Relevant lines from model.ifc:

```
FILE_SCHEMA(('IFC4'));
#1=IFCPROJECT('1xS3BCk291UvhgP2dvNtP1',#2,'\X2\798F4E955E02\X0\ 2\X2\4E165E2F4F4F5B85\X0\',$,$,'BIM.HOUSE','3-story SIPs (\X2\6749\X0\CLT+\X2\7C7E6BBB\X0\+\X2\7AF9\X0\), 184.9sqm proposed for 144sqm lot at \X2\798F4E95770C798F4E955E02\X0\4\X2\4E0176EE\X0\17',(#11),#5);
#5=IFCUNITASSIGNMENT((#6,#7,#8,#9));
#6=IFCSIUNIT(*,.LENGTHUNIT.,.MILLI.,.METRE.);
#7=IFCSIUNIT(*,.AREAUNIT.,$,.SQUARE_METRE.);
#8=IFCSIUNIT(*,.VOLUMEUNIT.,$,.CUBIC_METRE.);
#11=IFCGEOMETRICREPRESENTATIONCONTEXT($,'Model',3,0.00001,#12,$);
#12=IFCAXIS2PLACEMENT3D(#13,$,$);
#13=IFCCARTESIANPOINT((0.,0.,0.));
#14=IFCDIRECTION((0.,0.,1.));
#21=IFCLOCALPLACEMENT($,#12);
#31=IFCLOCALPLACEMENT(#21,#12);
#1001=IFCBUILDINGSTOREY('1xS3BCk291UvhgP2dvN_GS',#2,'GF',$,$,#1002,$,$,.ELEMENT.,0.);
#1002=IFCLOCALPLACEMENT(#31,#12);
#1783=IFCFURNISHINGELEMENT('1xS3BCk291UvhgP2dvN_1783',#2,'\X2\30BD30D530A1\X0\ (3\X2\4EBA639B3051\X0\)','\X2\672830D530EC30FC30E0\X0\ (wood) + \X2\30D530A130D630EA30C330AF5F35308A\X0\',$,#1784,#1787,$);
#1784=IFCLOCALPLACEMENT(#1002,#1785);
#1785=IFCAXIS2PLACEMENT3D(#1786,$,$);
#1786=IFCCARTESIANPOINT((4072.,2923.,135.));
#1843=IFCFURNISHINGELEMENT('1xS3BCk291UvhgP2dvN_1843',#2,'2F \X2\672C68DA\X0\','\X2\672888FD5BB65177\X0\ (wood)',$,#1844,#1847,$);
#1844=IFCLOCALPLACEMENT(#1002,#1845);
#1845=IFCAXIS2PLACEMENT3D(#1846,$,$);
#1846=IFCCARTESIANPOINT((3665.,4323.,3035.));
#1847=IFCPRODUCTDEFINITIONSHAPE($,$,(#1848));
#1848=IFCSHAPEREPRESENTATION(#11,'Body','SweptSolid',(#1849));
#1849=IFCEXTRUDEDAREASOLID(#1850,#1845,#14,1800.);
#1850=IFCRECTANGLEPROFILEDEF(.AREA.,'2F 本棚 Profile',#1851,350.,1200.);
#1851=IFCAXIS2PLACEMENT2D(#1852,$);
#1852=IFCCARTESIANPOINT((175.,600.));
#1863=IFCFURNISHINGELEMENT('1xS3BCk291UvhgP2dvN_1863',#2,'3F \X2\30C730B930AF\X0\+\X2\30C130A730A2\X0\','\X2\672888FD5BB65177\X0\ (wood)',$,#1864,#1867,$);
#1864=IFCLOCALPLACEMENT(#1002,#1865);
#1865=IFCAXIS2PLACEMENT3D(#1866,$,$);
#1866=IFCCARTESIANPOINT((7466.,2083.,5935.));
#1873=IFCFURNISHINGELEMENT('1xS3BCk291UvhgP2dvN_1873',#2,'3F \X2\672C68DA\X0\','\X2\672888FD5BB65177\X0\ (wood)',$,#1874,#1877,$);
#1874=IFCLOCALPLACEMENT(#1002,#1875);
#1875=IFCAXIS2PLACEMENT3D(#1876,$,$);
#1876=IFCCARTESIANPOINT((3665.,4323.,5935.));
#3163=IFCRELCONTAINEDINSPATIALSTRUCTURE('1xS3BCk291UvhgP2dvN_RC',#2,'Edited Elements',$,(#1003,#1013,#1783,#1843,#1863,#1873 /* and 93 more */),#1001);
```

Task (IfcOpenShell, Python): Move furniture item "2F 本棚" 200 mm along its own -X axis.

```python
import ifcopenshell
import ifcopenshell.api.geometry
import ifcopenshell.util.placement

model = ifcopenshell.open("model.ifc")

item = model.by_guid("1xS3BCk291UvhgP2dvN_1843")
matrix = ifcopenshell.util.placement.get_local_placement(item.ObjectPlacement)
matrix[:3, 3] -= matrix[:3, 0] * 200.0
ifcopenshell.api.geometry.edit_object_placement(model, product=item, matrix=matrix, is_si=False)

print(ifcopenshell.util.placement.get_local_placement(item.ObjectPlacement).round(3) + 0.0)

model.write("model_edited.ifc")
```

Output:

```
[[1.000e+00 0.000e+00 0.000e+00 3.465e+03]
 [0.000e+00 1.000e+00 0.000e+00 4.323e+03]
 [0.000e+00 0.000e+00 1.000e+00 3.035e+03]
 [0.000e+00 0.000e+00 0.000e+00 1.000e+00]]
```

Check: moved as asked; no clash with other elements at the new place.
